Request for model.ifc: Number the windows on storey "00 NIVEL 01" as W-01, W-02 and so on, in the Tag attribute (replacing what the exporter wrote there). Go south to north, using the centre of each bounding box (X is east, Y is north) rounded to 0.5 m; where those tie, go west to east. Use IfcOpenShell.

First a look at what the model holds.

```python
import ifcopenshell
import ifcopenshell.util.element
import ifcopenshell.util.placement

model = ifcopenshell.open("model.ifc")
print(model.schema)
storey = next(s for s in model.by_type("IfcBuildingStorey") if s.Name == "00 NIVEL 01")
windows = [e for e in ifcopenshell.util.element.get_decomposition(storey) if e.is_a("IfcWindow")]
for e in sorted(windows, key=lambda e: e.id()):
    origin = ifcopenshell.util.placement.get_local_placement(e.ObjectPlacement)[:3, 3]
    print(e.id(), e.Tag, e.Name, origin.round(2) + 0.0, sep=" | ")
```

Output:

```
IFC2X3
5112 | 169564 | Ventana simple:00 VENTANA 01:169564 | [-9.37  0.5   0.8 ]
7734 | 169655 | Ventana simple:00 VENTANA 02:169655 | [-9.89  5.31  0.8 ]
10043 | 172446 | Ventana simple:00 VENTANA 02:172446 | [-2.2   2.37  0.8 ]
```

```python
import ifcopenshell
import ifcopenshell.geom
import ifcopenshell.util.element
import ifcopenshell.util.shape

model = ifcopenshell.open("model.ifc")
settings = ifcopenshell.geom.settings()
settings.set("use-world-coords", True)


def centre(element):
    shape = ifcopenshell.geom.create_shape(settings, element)
    return ifcopenshell.util.shape.get_bbox_centroid(shape.geometry)


storey = next(s for s in model.by_type("IfcBuildingStorey") if s.Name == "00 NIVEL 01")
windows = [e for e in ifcopenshell.util.element.get_decomposition(storey) if e.is_a("IfcWindow")]

# Insertion points can sit at a corner or the storey origin, so sort by the geometry (in metres).
centres = {e: centre(e) for e in windows}
windows.sort(key=lambda e: (round(centres[e][1] / 0.5), centres[e][0]))

for i, e in enumerate(windows, start=1):
    number = f"W-{i:02d}"
    e.Tag = number
    print(e.id(), number)

model.write("model-out.ifc")
```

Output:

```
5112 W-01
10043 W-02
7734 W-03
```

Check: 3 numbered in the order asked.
